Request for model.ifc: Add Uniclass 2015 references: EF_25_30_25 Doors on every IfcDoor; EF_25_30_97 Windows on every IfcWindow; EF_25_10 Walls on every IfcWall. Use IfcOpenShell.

First a look at what the model holds.

```python
import ifcopenshell

model = ifcopenshell.open("model.ifc")
print(model.schema)
print("classifications:", [c.Name for c in model.by_type("IfcClassification")])
for ifc_class in ("IfcDoor", "IfcRoof", "IfcStair", "IfcWall", "IfcWindow"):
    print(ifc_class, len(model.by_type(ifc_class)))
```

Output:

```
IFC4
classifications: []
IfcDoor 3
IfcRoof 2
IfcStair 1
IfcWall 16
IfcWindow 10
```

```python
import ifcopenshell
import ifcopenshell.api.classification

model = ifcopenshell.open("model.ifc")

system = ifcopenshell.api.classification.add_classification(model, classification="Uniclass 2015")

codes = {
    "IfcDoor": ("EF_25_30_25", "Doors"),
    "IfcWindow": ("EF_25_30_97", "Windows"),
    "IfcWall": ("EF_25_10", "Walls"),
}
for ifc_class, (code, name) in codes.items():
    products = model.by_type(ifc_class)
    ifcopenshell.api.classification.add_reference(
        model, products=products, classification=system, identification=code, name=name
    )
    print(code, len(products))

model.write("model_rev.ifc")
```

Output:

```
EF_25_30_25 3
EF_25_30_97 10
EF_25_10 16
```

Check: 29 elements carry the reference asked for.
